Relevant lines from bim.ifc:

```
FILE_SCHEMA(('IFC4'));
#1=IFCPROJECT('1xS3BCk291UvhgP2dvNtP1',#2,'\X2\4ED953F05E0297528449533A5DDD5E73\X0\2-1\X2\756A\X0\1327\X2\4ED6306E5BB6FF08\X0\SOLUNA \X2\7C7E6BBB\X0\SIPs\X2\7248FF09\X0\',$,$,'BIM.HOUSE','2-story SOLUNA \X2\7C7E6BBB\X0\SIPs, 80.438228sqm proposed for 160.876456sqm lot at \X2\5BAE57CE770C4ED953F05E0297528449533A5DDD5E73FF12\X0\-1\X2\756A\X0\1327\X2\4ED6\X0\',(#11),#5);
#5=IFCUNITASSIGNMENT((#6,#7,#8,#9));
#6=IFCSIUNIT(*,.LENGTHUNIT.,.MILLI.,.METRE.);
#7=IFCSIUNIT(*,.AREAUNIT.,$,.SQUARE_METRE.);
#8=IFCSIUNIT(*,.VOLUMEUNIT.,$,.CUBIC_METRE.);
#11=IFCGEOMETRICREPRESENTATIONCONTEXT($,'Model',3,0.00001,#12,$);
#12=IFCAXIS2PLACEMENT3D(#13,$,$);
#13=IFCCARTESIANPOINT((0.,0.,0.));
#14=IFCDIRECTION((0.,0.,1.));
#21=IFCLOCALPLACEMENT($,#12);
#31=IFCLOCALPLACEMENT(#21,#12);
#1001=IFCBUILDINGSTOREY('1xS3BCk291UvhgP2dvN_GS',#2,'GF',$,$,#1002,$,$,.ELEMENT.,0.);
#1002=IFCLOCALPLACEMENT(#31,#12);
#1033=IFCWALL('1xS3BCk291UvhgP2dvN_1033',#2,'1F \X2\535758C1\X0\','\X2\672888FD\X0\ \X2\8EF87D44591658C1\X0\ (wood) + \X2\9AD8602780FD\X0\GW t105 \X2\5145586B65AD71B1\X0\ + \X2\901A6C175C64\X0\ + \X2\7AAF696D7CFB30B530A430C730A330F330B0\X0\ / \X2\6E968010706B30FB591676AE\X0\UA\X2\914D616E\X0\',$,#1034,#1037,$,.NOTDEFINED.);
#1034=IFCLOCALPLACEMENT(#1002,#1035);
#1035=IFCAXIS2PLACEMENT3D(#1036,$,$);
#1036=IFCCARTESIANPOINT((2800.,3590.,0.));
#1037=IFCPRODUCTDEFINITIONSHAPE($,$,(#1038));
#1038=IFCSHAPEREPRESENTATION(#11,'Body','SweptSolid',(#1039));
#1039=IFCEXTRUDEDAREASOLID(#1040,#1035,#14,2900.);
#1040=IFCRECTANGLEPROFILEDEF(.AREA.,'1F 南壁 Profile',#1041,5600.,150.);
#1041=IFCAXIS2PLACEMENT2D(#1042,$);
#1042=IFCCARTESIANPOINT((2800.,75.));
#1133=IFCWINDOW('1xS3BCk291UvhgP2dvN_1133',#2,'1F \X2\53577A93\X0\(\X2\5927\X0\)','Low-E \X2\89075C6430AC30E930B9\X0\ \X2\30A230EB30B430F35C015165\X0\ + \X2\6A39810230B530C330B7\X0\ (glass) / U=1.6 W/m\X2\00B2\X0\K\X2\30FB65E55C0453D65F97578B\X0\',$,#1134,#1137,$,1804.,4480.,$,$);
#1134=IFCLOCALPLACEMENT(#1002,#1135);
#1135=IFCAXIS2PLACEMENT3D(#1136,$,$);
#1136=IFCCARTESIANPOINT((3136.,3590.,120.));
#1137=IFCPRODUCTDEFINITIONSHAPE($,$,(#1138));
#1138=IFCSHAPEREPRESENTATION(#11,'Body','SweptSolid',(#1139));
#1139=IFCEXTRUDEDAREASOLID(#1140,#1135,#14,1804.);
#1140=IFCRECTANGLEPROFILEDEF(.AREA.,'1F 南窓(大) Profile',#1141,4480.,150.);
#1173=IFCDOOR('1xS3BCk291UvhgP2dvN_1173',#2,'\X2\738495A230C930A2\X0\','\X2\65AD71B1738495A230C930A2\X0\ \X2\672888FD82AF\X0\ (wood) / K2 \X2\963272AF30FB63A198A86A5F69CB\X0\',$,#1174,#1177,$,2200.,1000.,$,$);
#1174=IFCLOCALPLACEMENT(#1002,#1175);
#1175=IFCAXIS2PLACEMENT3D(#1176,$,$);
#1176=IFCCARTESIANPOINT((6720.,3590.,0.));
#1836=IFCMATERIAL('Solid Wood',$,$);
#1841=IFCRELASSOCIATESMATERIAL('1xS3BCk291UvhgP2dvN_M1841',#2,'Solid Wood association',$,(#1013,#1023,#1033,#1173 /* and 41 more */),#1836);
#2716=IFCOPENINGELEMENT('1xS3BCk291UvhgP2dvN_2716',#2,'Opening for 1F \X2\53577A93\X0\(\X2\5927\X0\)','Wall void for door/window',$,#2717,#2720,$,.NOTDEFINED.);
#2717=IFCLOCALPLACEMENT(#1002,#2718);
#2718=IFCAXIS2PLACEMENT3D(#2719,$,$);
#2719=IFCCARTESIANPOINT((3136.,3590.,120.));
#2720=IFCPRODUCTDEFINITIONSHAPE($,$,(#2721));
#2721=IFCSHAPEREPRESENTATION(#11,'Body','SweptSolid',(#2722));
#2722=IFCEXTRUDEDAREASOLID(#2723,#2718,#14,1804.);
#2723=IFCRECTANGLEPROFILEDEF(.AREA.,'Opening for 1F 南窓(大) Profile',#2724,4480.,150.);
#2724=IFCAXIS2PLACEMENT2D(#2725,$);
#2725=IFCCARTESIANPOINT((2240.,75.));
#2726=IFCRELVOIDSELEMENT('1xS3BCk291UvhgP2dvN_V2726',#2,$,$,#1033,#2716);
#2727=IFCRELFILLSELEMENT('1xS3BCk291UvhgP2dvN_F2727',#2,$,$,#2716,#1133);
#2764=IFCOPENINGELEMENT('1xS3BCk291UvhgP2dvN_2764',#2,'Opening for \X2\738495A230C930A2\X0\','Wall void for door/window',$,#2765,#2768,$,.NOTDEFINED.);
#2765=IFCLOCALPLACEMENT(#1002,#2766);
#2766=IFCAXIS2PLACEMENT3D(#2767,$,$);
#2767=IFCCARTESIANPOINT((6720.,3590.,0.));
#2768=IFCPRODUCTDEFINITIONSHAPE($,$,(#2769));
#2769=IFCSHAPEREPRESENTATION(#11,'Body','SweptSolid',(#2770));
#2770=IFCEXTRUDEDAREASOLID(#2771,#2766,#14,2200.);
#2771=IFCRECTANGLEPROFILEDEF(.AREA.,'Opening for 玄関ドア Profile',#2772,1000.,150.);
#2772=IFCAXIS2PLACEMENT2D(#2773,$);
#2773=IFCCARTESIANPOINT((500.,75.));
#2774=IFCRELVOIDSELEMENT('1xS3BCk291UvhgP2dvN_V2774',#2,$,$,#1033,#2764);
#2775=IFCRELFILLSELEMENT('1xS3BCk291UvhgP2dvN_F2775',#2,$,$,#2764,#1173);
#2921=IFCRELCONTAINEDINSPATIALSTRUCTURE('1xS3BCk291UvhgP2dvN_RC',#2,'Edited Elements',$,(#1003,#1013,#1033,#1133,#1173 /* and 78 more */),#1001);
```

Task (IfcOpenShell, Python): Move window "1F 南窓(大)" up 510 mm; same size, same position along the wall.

```python
import numpy as np
import ifcopenshell
import ifcopenshell.api.geometry
import ifcopenshell.util.placement
import ifcopenshell.util.unit

model = ifcopenshell.open("bim.ifc")
unit_scale = ifcopenshell.util.unit.calculate_unit_scale(model)

window = model.by_id(1133)
opening = window.FillsVoids[0].RelatingOpeningElement
dz = 510.0

shift = np.array([0.0, 0.0, dz])
# The window is not placed relative to its opening, so move both.
for product in (opening, window):
    matrix = ifcopenshell.util.placement.get_local_placement(product.ObjectPlacement)
    matrix[:3, 3] += shift
    ifcopenshell.api.geometry.edit_object_placement(model, product=product, matrix=matrix, is_si=False)

print(f"moved by {dz * unit_scale:+.3f} m")

model.write("bim_rev.ifc")
```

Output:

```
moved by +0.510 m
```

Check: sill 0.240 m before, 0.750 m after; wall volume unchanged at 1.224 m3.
